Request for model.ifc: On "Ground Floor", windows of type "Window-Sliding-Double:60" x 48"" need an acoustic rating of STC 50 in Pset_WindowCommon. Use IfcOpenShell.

First a look at what the model holds.

```python
import ifcopenshell
import ifcopenshell.util.element

model = ifcopenshell.open("model.ifc")
print(model.schema)
storey = next(s for s in model.by_type("IfcBuildingStorey") if s.Name == "Ground Floor")
windows = [e for e in ifcopenshell.util.element.get_decomposition(storey) if e.is_a("IfcWindow")]
seen = {}
for e in windows:
    element_type = ifcopenshell.util.element.get_type(e)
    key = (element_type.Name if element_type != e and element_type else None, ifcopenshell.util.element.get_pset(e, "Pset_WindowCommon", "AcousticRating"))
    seen[key] = seen.get(key, 0) + 1
for (name, value), count in sorted(seen.items(), key=str):
    print(count, "x", name, "|", value)
```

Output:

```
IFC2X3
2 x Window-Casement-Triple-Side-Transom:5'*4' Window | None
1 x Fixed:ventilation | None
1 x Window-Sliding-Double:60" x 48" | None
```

```python
import ifcopenshell
import ifcopenshell.api.pset
import ifcopenshell.util.element

model = ifcopenshell.open("model.ifc")

storey = next(s for s in model.by_type("IfcBuildingStorey") if s.Name == "Ground Floor")
windows = [e for e in ifcopenshell.util.element.get_decomposition(storey) if e.is_a("IfcWindow")]

count = 0
for e in windows:
    element_type = ifcopenshell.util.element.get_type(e)
    if element_type in (None, e) or element_type.Name != 'Window-Sliding-Double:60" x 48"':
        continue
    # add_pset returns the element's existing set when there is one.
    pset = ifcopenshell.api.pset.add_pset(model, product=e, name="Pset_WindowCommon")
    ifcopenshell.api.pset.edit_pset(model, pset=pset, properties={"AcousticRating": "STC 50"})
    count += 1

print(count, "windows updated")

model.write("model_updated.ifc")
```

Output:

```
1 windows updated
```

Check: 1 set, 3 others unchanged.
